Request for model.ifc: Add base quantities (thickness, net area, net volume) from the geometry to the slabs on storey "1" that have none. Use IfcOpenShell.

First a look at what the model holds.

```python
import ifcopenshell
import ifcopenshell.util.element
import ifcopenshell.util.unit

model = ifcopenshell.open("model.ifc")
print(model.schema)
for unit_type in ("LENGTHUNIT", "AREAUNIT", "VOLUMEUNIT"):
    print(unit_type, ifcopenshell.util.unit.calculate_unit_scale(model, unit_type))
storey = next(s for s in model.by_type("IfcBuildingStorey") if s.Name == "1")
slabs = [e for e in ifcopenshell.util.element.get_decomposition(storey) if e.is_a("IfcSlab")]
for e in sorted(slabs, key=lambda e: e.id()):
    print(e.id(), e.is_a(), e.Name, list(ifcopenshell.util.element.get_psets(e, qtos_only=True)), sep=" | ")
```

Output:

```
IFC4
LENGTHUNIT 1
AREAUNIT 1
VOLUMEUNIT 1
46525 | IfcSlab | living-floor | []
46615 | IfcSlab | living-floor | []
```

```python
import ifcopenshell
import ifcopenshell.api.pset
import ifcopenshell.geom
import ifcopenshell.util.element
import ifcopenshell.util.shape
import ifcopenshell.util.unit

model = ifcopenshell.open("model.ifc")
unit_scale = ifcopenshell.util.unit.calculate_unit_scale(model)
area_scale = ifcopenshell.util.unit.calculate_unit_scale(model, "AREAUNIT")
volume_scale = ifcopenshell.util.unit.calculate_unit_scale(model, "VOLUMEUNIT")
settings = ifcopenshell.geom.settings()

storey = next(s for s in model.by_type("IfcBuildingStorey") if s.Name == "1")
slabs = [e for e in ifcopenshell.util.element.get_decomposition(storey) if e.is_a("IfcSlab")]

for e in sorted(slabs, key=lambda e: e.id()):
    if ifcopenshell.util.element.get_psets(e, qtos_only=True, should_inherit=False):
        continue
    # Geometry comes back in metres, in the element's own axes.
    shape = ifcopenshell.geom.create_shape(settings, e)
    values = {
        "Width": ifcopenshell.util.shape.get_z(shape.geometry) / unit_scale,
        "NetArea": ifcopenshell.util.shape.get_footprint_area(shape.geometry) / area_scale,
        "NetVolume": ifcopenshell.util.shape.get_volume(shape.geometry) / volume_scale,
    }
    qto = ifcopenshell.api.pset.add_qto(model, product=e, name="Qto_SlabBaseQuantities")
    ifcopenshell.api.pset.edit_qto(model, qto=qto, properties=values)
    print(e.id(), {k: round(v, 3) for k, v in values.items()})

model.write("model-out.ifc")
```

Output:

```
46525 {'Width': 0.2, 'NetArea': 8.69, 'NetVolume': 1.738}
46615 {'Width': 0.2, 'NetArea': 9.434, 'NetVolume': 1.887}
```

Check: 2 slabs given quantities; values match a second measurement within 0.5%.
